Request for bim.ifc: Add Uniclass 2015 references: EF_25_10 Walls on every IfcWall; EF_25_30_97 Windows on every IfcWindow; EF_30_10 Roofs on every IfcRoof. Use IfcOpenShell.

First a look at what the model holds.

```python
import ifcopenshell

model = ifcopenshell.open("bim.ifc")
print(model.schema)
print("classifications:", [c.Name for c in model.by_type("IfcClassification")])
for ifc_class in ("IfcDoor", "IfcRoof", "IfcStair", "IfcWall", "IfcWindow"):
    print(ifc_class, len(model.by_type(ifc_class)))
```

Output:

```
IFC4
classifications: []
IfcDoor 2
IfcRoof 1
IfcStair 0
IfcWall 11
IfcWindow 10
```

```python
import ifcopenshell
import ifcopenshell.api.classification

model = ifcopenshell.open("bim.ifc")

system = ifcopenshell.api.classification.add_classification(model, classification="Uniclass 2015")

codes = {
    "IfcWall": ("EF_25_10", "Walls"),
    "IfcWindow": ("EF_25_30_97", "Windows"),
    "IfcRoof": ("EF_30_10", "Roofs"),
}
for ifc_class, (code, name) in codes.items():
    products = model.by_type(ifc_class)
    ifcopenshell.api.classification.add_reference(
        model, products=products, classification=system, identification=code, name=name
    )
    print(code, len(products))

model.write("bim-out.ifc")
```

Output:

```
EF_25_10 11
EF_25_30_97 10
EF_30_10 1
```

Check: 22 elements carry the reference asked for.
